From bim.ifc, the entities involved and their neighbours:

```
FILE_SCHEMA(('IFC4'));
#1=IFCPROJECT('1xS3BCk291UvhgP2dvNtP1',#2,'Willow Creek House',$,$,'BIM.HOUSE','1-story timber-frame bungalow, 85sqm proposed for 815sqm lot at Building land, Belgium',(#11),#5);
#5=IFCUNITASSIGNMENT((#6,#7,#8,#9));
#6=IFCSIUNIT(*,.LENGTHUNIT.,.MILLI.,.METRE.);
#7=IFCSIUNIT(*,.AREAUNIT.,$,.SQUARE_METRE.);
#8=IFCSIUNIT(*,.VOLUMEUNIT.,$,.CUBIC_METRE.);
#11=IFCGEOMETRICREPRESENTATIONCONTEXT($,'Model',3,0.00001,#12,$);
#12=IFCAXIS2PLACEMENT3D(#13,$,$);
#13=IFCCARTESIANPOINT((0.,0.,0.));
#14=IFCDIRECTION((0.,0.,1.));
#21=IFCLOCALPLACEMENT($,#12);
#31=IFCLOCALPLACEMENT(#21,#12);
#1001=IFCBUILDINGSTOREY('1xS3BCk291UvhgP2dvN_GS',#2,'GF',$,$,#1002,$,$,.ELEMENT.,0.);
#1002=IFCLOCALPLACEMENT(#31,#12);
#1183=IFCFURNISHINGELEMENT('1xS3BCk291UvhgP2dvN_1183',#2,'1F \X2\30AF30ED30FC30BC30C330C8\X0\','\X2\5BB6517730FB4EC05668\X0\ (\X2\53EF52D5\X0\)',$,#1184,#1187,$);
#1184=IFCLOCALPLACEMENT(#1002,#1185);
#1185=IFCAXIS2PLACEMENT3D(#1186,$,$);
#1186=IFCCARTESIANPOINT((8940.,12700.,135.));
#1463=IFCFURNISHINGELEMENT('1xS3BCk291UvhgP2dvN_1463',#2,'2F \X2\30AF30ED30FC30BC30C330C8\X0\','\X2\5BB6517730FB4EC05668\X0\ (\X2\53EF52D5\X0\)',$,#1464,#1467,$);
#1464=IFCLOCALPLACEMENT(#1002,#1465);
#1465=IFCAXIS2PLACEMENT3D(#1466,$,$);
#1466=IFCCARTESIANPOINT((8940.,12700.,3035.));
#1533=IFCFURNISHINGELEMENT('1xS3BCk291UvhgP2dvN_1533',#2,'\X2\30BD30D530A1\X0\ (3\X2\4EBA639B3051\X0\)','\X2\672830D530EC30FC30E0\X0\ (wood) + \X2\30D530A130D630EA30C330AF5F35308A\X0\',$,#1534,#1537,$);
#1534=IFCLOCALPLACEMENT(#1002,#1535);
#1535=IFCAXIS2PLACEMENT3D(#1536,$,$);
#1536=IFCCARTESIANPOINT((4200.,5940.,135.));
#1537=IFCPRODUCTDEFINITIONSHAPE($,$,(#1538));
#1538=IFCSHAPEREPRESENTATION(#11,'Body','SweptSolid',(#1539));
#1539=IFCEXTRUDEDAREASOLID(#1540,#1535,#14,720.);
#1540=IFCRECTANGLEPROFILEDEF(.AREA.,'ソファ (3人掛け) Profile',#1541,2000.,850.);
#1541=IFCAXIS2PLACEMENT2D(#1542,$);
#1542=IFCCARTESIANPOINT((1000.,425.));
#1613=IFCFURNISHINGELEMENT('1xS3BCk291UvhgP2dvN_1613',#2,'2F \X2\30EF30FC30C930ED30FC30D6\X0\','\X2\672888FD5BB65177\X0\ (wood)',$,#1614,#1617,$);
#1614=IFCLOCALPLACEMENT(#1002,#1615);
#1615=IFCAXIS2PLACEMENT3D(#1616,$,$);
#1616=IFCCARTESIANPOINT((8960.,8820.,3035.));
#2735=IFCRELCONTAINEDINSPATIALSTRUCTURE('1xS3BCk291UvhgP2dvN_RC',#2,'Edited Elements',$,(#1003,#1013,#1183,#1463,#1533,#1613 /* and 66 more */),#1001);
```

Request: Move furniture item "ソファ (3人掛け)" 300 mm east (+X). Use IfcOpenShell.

```python
import ifcopenshell
import ifcopenshell.api.geometry
import ifcopenshell.util.placement
import ifcopenshell.util.unit

model = ifcopenshell.open("bim.ifc")
unit_scale = ifcopenshell.util.unit.calculate_unit_scale(model)

item = model.by_guid("1xS3BCk291UvhgP2dvN_1533")
matrix = ifcopenshell.util.placement.get_local_placement(item.ObjectPlacement)
matrix[0, 3] += 0.3 / unit_scale
ifcopenshell.api.geometry.edit_object_placement(model, product=item, matrix=matrix, is_si=False)

print(ifcopenshell.util.placement.get_local_placement(item.ObjectPlacement).round(3) + 0.0)

model.write("bim-out.ifc")
```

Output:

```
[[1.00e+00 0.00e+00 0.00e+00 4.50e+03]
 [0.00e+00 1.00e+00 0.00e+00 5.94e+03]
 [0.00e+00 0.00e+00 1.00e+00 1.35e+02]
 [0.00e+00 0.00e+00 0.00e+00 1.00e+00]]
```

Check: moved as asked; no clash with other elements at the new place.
